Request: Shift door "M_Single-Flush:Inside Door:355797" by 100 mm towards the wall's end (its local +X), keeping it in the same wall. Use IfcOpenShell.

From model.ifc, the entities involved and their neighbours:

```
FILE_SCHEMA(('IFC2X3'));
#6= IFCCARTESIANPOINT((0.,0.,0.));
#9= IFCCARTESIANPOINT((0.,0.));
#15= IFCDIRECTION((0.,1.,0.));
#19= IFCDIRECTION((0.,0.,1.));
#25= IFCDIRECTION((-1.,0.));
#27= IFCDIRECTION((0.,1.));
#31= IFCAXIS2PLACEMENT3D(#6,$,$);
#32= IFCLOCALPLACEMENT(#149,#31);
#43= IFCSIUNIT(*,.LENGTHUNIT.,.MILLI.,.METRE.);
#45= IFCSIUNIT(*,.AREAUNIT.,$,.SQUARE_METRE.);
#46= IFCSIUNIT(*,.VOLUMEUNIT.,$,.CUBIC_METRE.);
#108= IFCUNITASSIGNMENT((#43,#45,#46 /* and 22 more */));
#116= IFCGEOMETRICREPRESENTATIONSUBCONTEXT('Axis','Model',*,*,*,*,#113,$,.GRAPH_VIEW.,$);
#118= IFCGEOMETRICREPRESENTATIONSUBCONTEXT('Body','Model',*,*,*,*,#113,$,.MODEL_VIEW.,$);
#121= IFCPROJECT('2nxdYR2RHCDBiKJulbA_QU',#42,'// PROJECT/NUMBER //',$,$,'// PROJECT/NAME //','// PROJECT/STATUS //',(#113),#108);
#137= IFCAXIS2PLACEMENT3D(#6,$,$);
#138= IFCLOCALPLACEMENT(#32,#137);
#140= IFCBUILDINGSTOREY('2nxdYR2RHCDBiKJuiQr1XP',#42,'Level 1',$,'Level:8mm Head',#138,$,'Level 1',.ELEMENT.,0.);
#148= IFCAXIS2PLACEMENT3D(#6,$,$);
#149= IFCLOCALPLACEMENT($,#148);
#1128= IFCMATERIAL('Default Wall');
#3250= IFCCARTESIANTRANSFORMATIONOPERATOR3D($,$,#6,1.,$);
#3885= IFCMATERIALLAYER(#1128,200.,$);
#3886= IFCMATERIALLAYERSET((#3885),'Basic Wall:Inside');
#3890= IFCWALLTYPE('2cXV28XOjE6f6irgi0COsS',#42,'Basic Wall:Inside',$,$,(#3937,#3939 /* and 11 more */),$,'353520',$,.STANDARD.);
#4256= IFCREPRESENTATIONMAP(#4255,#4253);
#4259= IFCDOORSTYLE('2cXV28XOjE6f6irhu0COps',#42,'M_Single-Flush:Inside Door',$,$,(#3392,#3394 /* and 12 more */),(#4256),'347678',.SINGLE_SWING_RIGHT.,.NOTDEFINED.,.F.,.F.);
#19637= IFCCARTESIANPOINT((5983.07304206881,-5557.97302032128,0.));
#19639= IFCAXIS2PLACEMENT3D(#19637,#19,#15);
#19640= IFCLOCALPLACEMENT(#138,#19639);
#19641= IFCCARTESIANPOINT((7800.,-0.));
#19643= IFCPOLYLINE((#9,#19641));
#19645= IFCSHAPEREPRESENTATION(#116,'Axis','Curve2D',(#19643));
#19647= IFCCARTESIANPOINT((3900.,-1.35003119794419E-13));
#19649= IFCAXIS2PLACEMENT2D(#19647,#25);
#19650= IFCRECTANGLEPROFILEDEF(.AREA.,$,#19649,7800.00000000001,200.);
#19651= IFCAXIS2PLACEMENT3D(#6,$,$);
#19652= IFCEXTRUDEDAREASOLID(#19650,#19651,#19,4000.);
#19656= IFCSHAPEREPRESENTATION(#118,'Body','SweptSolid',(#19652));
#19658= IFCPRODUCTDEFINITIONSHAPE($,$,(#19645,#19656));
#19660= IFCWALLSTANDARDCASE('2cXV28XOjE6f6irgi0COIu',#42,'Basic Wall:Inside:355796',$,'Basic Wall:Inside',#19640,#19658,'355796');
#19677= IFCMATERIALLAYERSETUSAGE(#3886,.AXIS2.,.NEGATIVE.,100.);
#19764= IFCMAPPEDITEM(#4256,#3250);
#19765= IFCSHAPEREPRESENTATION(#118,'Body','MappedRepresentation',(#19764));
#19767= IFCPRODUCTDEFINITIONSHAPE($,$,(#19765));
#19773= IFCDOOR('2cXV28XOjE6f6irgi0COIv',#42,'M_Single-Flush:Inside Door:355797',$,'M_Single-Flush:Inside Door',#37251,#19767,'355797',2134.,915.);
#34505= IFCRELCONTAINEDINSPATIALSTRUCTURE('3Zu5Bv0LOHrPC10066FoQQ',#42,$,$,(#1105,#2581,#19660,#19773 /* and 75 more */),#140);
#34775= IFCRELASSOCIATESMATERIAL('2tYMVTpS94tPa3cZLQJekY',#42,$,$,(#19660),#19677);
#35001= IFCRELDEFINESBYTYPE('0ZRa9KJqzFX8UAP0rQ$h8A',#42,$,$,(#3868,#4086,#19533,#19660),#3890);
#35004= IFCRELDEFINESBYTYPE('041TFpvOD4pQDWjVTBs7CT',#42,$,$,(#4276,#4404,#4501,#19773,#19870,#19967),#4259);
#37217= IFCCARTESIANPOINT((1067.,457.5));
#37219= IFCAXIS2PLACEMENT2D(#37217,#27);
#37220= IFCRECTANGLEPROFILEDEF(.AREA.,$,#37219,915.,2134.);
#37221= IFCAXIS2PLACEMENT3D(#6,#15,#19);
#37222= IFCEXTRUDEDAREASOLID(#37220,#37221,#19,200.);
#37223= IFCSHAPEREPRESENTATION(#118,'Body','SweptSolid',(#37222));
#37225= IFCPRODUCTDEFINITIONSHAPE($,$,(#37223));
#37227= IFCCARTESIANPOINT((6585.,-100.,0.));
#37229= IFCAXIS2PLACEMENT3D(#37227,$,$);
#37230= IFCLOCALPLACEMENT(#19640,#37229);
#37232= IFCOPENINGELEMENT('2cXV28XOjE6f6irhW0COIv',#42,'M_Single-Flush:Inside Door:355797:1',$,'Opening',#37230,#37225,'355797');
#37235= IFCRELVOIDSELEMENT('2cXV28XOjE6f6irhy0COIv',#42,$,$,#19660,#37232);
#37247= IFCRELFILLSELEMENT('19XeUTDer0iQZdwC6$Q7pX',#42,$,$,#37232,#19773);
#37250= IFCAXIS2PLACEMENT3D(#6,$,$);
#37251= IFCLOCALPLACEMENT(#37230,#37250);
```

```python
import ifcopenshell
import ifcopenshell.api.geometry
import ifcopenshell.util.placement
import ifcopenshell.util.unit

model = ifcopenshell.open("model.ifc")
unit_scale = ifcopenshell.util.unit.calculate_unit_scale(model)

door = model.by_guid("2cXV28XOjE6f6irgi0COIv")
opening = door.FillsVoids[0].RelatingOpeningElement
wall = opening.VoidsElements[0].RelatingBuildingElement

wall_matrix = ifcopenshell.util.placement.get_local_placement(wall.ObjectPlacement)
shift = wall_matrix[:3, 0] * 0.1 / unit_scale
before = ifcopenshell.util.placement.get_local_placement(door.ObjectPlacement)[:3, 3].copy()

# The door is placed relative to its opening, so it follows when the opening moves.
matrix = ifcopenshell.util.placement.get_local_placement(opening.ObjectPlacement)
matrix[:3, 3] += shift
ifcopenshell.api.geometry.edit_object_placement(
    model, product=opening, matrix=matrix, is_si=False, should_transform_children=True
)

after = ifcopenshell.util.placement.get_local_placement(door.ObjectPlacement)[:3, 3]
print("door moved by", (after - before).round(3) + 0.0)

model.write("model_rev.ifc")
```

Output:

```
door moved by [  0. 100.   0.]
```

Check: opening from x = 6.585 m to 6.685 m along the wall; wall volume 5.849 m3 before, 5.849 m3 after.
